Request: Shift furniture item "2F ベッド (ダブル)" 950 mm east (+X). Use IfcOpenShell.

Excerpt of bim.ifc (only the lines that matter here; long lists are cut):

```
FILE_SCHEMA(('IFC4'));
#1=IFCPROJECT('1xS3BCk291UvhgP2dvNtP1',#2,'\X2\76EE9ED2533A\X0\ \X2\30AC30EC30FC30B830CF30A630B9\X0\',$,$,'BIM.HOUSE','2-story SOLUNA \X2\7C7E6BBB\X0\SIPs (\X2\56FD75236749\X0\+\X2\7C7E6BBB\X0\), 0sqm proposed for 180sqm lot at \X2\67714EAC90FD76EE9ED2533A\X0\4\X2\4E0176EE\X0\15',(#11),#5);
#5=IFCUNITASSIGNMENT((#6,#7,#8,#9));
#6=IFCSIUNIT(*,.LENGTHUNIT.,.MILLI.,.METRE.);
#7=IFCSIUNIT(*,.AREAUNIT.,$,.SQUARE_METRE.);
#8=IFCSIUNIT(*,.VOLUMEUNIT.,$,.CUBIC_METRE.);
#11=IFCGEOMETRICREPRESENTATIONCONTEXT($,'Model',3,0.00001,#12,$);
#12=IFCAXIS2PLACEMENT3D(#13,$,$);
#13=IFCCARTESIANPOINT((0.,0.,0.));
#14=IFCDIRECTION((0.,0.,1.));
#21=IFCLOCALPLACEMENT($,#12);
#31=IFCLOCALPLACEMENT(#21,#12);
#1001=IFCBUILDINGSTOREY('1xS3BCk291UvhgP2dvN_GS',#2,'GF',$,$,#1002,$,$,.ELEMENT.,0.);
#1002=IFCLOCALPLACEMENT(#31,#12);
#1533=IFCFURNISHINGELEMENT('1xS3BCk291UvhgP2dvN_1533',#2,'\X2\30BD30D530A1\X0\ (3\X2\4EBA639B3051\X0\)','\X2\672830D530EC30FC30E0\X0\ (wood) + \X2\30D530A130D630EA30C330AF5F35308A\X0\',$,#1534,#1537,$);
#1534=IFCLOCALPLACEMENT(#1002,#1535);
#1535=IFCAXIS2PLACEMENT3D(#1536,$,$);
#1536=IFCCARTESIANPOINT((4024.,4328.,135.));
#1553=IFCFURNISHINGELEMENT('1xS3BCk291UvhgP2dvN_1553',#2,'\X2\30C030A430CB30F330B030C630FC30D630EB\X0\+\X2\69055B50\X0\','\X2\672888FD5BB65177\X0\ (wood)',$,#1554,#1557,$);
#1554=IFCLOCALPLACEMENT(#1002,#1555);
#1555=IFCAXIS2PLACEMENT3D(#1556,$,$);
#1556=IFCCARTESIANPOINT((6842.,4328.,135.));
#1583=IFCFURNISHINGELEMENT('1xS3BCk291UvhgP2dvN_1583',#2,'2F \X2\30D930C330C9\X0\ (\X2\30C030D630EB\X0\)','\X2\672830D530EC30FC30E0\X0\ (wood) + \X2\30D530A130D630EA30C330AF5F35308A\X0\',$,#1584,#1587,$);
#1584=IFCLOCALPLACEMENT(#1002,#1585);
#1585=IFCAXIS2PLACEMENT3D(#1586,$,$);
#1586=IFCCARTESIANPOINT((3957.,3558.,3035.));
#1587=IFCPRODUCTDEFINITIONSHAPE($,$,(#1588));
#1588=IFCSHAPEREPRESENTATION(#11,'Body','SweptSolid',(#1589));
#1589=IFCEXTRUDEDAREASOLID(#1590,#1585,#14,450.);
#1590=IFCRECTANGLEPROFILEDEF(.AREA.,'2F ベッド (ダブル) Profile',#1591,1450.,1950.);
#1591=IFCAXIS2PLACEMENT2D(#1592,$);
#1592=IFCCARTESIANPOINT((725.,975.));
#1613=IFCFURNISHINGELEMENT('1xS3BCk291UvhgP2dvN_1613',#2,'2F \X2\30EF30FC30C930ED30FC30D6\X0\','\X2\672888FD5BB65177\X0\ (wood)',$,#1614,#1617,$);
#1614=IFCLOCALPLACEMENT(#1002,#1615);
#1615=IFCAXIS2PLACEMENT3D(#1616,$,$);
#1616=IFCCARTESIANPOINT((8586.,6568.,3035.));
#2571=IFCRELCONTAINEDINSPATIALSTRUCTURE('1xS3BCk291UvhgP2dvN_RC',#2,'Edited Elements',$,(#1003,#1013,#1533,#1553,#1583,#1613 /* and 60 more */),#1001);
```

```python
import ifcopenshell
import ifcopenshell.api.geometry
import ifcopenshell.util.placement

model = ifcopenshell.open("bim.ifc")

item = model.by_guid("1xS3BCk291UvhgP2dvN_1583")
matrix = ifcopenshell.util.placement.get_local_placement(item.ObjectPlacement)
matrix[0, 3] += 950.0
ifcopenshell.api.geometry.edit_object_placement(model, product=item, matrix=matrix, is_si=False)

print(ifcopenshell.util.placement.get_local_placement(item.ObjectPlacement).round(3) + 0.0)

model.write("bim-out.ifc")
```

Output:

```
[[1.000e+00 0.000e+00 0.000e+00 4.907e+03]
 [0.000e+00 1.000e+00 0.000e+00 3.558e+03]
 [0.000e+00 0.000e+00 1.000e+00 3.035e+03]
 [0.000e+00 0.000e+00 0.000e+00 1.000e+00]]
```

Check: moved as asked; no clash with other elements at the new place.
